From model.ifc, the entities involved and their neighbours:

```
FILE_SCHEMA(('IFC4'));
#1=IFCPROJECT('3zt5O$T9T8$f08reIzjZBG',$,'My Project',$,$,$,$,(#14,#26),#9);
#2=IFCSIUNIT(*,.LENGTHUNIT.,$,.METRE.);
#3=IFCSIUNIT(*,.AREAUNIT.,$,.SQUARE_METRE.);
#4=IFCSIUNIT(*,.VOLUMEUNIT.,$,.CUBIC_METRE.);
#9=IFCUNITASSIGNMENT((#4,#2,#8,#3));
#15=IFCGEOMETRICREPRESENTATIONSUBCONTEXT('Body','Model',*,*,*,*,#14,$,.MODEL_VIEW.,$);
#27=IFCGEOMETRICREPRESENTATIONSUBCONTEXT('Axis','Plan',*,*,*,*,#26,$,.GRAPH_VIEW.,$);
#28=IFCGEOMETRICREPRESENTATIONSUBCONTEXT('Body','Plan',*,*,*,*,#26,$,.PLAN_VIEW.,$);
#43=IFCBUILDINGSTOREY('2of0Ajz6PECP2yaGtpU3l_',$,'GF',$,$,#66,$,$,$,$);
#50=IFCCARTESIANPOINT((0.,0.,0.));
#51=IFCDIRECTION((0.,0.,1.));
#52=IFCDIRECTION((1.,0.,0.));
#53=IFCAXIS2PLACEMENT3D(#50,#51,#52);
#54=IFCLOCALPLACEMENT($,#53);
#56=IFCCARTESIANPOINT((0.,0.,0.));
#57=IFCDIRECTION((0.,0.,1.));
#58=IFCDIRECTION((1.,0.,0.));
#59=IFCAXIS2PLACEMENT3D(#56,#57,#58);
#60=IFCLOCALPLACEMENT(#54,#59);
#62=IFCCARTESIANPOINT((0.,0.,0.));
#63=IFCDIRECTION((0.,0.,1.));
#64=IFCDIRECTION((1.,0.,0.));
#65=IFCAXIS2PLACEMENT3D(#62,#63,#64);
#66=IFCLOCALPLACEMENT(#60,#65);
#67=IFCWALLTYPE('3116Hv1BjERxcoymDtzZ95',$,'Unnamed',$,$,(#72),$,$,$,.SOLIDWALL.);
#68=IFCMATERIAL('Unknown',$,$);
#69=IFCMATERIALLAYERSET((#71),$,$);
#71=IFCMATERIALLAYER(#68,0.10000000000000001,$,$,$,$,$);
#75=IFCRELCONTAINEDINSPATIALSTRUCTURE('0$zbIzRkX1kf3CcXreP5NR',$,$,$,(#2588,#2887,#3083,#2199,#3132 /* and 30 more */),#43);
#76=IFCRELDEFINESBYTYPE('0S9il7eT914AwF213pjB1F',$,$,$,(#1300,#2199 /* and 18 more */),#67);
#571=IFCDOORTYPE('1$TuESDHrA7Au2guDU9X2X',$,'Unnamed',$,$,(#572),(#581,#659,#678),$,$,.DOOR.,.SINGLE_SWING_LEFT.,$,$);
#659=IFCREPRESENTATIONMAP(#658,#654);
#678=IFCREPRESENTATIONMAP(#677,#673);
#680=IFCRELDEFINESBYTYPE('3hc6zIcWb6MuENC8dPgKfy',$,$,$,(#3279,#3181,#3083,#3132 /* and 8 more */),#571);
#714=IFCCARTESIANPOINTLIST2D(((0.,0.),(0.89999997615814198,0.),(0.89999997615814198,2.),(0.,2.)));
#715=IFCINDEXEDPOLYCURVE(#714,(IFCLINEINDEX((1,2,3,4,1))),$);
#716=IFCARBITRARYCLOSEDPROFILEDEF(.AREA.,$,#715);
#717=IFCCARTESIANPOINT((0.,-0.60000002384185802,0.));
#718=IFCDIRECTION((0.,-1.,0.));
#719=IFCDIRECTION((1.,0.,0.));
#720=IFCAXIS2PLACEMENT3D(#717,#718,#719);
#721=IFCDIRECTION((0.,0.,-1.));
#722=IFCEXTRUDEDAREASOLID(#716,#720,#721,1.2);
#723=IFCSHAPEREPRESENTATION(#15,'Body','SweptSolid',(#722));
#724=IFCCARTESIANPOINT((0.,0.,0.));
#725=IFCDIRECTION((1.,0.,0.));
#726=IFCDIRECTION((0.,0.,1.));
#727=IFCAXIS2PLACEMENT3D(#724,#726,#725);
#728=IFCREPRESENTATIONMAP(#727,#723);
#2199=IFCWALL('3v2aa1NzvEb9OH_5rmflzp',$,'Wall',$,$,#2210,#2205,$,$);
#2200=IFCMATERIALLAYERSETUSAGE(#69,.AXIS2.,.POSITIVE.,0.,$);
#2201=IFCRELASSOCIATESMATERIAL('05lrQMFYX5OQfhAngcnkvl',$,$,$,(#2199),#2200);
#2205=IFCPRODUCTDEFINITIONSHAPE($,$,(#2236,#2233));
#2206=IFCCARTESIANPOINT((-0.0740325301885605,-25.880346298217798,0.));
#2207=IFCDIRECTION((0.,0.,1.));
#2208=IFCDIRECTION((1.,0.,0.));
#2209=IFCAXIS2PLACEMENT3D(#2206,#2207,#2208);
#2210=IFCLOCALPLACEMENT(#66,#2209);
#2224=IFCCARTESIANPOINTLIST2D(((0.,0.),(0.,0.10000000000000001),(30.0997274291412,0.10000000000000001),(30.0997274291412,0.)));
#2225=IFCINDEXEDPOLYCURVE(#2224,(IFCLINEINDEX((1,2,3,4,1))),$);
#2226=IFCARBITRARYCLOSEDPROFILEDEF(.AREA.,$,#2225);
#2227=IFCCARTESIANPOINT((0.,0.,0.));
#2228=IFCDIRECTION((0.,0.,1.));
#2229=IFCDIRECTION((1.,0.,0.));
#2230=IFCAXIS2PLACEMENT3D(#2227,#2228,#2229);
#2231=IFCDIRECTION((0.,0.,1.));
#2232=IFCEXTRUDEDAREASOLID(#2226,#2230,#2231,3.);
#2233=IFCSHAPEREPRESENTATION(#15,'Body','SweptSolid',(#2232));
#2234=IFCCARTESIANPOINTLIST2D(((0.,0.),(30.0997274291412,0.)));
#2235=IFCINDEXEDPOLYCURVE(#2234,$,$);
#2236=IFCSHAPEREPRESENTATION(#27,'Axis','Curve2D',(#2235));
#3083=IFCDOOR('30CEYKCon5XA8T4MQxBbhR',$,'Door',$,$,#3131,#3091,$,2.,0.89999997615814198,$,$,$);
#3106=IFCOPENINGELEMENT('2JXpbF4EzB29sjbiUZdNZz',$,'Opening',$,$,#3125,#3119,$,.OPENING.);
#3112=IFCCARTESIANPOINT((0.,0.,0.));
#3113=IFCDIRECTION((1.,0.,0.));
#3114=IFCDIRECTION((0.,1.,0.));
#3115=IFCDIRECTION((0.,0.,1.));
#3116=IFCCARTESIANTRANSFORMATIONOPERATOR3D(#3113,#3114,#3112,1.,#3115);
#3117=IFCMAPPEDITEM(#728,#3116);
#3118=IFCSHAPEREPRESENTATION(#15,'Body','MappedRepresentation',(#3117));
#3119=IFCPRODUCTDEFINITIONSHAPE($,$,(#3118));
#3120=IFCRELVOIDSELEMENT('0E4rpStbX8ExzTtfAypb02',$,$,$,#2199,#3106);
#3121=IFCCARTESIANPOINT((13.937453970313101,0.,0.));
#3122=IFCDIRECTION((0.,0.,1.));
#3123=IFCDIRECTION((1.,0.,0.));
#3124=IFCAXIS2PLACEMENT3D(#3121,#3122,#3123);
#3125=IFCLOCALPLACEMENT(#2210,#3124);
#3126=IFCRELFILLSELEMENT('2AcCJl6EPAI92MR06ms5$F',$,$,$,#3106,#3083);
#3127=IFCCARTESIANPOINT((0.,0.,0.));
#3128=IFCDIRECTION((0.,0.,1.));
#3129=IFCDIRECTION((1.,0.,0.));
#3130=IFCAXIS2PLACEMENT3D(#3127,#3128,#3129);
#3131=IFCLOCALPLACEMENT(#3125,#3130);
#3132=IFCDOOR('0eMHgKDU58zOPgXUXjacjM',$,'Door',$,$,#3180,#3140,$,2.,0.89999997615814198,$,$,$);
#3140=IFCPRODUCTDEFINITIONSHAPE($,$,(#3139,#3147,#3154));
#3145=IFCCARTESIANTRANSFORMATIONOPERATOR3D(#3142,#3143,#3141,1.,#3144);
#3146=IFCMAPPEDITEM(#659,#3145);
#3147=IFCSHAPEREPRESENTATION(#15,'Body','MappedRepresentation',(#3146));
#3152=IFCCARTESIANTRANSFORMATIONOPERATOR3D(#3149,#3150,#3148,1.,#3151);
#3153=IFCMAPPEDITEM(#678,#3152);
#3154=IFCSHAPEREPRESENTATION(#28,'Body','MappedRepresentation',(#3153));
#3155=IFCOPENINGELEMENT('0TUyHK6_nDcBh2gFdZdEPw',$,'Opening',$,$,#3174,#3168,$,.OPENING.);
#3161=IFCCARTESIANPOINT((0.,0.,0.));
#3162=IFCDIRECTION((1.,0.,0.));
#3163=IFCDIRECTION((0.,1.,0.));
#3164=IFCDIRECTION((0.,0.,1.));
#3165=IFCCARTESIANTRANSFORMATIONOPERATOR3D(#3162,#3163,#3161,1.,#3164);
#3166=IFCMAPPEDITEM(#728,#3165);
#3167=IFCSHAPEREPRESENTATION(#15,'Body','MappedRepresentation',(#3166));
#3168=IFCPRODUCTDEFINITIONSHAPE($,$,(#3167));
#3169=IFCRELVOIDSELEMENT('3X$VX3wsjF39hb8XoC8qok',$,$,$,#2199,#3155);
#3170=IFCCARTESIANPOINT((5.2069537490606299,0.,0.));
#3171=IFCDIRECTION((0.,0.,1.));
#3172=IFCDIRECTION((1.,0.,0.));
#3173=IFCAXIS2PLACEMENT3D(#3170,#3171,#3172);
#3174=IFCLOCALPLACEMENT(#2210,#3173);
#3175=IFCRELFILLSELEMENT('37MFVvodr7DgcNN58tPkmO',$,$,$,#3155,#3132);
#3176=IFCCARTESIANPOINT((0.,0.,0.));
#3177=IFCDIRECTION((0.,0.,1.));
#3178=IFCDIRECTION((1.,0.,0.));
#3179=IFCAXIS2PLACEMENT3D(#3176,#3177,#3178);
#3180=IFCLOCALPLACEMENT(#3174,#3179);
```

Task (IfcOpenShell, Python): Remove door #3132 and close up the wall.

```python
import ifcopenshell
import ifcopenshell.api.feature
import ifcopenshell.api.root
import ifcopenshell.geom
import ifcopenshell.util.shape

model = ifcopenshell.open("model.ifc")
settings = ifcopenshell.geom.settings()


def volume(element):
    """Net volume in cubic metres, openings subtracted."""
    shape = ifcopenshell.geom.create_shape(settings, element)
    return ifcopenshell.util.shape.get_volume(shape.geometry)


door = model.by_guid("0eMHgKDU58zOPgXUXjacjM")
opening = door.FillsVoids[0].RelatingOpeningElement
wall = opening.VoidsElements[0].RelatingBuildingElement
before = volume(wall)

ifcopenshell.api.root.remove_product(model, product=door)
ifcopenshell.api.feature.remove_feature(model, feature=opening)

after = volume(wall)

print(f"wall volume {before:.3f} -> {after:.3f} m3")

model.write("model_updated.ifc")
```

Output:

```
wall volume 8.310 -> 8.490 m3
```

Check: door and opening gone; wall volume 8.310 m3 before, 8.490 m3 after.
